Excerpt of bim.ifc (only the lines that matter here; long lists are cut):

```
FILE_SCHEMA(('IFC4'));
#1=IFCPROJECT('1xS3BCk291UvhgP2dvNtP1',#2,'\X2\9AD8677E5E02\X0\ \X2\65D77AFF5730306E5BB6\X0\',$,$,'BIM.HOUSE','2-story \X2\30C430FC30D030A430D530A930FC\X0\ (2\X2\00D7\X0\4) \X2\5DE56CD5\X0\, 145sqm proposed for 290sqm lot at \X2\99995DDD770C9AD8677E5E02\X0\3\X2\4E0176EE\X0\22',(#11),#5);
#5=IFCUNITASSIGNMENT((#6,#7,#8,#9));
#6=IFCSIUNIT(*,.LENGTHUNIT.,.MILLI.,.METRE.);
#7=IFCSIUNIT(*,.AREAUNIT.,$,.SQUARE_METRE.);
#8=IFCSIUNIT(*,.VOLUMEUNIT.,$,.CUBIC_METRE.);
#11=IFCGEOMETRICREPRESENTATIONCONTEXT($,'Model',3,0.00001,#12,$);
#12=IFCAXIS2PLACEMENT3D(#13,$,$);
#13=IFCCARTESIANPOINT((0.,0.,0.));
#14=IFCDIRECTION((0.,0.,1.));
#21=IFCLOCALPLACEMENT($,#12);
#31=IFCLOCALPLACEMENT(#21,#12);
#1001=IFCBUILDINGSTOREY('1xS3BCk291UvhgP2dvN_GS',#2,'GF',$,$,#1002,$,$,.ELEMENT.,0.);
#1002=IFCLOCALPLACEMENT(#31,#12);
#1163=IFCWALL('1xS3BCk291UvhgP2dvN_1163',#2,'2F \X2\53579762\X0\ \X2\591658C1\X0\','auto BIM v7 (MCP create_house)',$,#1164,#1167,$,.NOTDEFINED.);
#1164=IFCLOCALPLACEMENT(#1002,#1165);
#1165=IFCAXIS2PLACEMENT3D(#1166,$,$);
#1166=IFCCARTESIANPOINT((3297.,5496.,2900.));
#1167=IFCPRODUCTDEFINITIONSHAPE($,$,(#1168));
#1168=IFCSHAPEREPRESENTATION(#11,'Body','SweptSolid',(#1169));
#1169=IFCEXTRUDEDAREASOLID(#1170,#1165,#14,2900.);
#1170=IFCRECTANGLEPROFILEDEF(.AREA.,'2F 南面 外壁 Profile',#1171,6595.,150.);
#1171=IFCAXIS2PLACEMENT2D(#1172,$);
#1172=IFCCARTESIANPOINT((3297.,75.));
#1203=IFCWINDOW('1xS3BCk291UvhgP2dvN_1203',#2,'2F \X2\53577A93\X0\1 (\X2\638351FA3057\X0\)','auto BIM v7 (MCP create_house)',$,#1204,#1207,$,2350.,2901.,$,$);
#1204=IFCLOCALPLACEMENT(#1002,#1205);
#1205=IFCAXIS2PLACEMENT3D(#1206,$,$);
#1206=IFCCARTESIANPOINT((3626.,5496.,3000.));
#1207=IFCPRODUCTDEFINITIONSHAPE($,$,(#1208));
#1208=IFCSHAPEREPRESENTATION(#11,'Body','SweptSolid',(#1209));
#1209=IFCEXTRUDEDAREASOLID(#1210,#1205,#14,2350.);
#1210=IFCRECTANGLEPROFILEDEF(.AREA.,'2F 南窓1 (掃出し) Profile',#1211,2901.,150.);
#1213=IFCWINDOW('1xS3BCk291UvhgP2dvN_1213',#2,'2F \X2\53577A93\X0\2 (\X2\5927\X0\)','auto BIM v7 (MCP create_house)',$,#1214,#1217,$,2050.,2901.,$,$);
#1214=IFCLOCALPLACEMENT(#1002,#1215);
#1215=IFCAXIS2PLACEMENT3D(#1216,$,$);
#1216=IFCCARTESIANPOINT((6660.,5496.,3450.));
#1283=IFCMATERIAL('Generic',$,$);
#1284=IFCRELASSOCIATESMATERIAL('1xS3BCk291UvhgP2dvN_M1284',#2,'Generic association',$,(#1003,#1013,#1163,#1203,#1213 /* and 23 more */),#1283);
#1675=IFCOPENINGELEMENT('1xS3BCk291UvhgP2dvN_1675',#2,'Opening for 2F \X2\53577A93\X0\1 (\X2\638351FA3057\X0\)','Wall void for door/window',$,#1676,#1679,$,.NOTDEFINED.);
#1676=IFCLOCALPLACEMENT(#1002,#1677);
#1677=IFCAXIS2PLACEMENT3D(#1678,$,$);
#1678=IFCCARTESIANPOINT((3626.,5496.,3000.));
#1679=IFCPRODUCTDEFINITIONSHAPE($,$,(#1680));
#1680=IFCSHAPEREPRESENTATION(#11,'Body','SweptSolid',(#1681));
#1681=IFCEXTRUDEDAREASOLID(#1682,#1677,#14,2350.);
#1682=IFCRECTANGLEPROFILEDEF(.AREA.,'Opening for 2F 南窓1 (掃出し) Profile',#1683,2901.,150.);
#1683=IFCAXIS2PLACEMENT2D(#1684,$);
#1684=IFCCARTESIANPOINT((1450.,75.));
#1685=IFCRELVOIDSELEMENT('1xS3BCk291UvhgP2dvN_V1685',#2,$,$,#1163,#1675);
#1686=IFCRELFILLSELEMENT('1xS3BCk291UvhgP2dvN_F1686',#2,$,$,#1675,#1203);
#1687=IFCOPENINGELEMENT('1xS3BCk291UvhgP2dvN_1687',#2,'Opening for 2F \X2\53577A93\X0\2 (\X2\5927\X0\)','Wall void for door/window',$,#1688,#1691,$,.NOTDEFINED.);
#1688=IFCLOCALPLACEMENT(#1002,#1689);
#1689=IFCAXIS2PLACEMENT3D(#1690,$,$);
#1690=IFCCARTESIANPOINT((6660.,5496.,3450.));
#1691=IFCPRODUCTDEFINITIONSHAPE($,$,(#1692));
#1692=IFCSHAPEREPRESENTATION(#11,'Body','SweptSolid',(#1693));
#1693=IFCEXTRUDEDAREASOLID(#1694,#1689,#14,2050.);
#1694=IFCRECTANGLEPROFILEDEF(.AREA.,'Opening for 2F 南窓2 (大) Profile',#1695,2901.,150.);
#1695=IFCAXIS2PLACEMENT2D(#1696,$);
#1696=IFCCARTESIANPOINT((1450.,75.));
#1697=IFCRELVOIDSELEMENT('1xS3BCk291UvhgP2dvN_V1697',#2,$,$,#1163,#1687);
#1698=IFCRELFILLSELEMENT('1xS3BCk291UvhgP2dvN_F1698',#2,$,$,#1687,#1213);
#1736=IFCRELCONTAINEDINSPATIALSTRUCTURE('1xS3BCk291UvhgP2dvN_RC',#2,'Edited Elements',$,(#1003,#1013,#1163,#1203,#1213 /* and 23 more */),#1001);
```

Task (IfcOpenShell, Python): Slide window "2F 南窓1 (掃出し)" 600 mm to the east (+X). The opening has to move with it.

```python
import ifcopenshell
import ifcopenshell.api.geometry
import ifcopenshell.util.placement
import ifcopenshell.util.unit

model = ifcopenshell.open("bim.ifc")
unit_scale = ifcopenshell.util.unit.calculate_unit_scale(model)

window = model.by_guid("1xS3BCk291UvhgP2dvN_1203")
opening = window.FillsVoids[0].RelatingOpeningElement
wall = opening.VoidsElements[0].RelatingBuildingElement

wall_matrix = ifcopenshell.util.placement.get_local_placement(wall.ObjectPlacement)
shift = wall_matrix[:3, 0] * 0.6 / unit_scale
before = ifcopenshell.util.placement.get_local_placement(window.ObjectPlacement)[:3, 3].copy()

# The window is not placed relative to its opening, so move both.
for product in (opening, window):
    matrix = ifcopenshell.util.placement.get_local_placement(product.ObjectPlacement)
    matrix[:3, 3] += shift
    ifcopenshell.api.geometry.edit_object_placement(model, product=product, matrix=matrix, is_si=False)

after = ifcopenshell.util.placement.get_local_placement(window.ObjectPlacement)[:3, 3]
print("window moved by", (after - before).round(3) + 0.0)

model.write("bim-out.ifc")
```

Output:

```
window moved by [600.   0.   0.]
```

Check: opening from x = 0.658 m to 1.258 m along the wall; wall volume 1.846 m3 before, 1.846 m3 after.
